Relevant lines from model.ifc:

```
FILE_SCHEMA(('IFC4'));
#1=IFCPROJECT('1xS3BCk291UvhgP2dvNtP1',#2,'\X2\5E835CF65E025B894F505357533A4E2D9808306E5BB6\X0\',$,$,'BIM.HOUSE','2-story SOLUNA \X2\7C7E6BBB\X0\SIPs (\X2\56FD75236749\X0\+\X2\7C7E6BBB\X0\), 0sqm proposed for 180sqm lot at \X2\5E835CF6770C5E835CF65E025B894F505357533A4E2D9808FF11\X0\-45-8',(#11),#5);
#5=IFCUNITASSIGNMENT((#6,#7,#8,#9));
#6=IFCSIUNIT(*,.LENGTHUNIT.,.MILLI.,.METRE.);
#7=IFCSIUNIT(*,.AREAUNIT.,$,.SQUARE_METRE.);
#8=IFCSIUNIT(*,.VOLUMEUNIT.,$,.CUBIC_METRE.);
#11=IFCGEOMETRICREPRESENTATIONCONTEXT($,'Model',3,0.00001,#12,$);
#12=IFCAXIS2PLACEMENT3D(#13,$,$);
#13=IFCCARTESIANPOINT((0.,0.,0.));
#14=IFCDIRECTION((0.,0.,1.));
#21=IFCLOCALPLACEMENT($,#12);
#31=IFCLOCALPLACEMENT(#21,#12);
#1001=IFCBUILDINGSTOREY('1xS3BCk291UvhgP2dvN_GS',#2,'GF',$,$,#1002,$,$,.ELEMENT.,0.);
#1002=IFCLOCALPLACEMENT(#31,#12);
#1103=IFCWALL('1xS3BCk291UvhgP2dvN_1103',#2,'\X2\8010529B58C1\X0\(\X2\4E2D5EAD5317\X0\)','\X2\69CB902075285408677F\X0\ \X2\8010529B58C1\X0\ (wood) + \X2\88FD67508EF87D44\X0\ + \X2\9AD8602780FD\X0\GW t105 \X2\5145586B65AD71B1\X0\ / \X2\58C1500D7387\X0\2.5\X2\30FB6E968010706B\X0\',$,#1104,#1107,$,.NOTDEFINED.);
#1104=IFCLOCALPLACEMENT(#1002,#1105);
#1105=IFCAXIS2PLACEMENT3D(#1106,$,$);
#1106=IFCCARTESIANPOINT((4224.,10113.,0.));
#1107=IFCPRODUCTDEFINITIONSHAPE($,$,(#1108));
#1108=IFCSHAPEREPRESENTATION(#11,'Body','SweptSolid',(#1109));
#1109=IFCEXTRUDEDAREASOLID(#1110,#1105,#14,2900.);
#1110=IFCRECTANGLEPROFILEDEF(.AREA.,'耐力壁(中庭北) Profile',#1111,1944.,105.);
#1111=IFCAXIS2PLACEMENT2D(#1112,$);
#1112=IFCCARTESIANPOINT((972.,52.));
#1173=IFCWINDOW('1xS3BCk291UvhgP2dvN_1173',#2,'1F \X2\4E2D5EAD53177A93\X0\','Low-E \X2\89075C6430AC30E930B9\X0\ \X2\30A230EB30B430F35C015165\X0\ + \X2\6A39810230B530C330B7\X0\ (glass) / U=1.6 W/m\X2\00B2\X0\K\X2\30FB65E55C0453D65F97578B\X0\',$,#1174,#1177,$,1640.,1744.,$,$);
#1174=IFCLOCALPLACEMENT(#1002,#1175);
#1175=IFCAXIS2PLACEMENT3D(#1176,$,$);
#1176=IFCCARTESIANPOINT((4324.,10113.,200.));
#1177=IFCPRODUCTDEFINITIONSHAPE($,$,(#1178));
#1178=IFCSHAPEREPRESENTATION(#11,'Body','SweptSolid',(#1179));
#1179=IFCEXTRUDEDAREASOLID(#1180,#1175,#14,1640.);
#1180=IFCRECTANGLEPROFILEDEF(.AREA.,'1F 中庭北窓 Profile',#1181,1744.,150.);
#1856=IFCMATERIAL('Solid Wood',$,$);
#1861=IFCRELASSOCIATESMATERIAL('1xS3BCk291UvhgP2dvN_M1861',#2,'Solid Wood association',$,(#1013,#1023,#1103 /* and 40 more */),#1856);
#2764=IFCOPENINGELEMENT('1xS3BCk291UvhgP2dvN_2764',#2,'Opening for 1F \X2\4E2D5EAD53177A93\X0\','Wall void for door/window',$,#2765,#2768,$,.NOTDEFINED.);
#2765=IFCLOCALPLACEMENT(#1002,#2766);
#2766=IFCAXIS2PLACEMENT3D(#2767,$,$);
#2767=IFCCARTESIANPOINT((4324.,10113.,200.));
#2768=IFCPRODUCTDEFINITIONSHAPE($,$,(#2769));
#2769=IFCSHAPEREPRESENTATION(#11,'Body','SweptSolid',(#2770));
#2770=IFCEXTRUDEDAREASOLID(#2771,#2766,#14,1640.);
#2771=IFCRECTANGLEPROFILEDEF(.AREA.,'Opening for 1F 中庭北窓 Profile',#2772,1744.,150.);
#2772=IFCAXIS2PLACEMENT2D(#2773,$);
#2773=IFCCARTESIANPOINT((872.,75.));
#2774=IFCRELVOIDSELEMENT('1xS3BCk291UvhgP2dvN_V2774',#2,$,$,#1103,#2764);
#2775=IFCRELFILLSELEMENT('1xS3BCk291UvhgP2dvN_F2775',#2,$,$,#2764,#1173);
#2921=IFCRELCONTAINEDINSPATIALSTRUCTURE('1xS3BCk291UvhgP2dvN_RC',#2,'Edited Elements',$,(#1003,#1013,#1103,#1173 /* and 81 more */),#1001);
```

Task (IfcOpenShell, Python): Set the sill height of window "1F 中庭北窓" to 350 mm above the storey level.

```python
import numpy as np
import ifcopenshell
import ifcopenshell.api.geometry
import ifcopenshell.geom
import ifcopenshell.util.element
import ifcopenshell.util.placement
import ifcopenshell.util.shape
import ifcopenshell.util.unit

model = ifcopenshell.open("model.ifc")
unit_scale = ifcopenshell.util.unit.calculate_unit_scale(model)

window = model.by_id(1173)
opening = window.FillsVoids[0].RelatingOpeningElement
storey = ifcopenshell.util.element.get_container(window, ifc_class="IfcBuildingStorey")
level = ifcopenshell.util.placement.get_local_placement(storey.ObjectPlacement)[2, 3]

# The opening's origin need not be at the sill, so measure its lowest point.
shape = ifcopenshell.geom.create_shape(ifcopenshell.geom.settings(), opening)
bottom = ifcopenshell.util.shape.get_shape_bottom_elevation(shape, shape.geometry) / unit_scale
dz = level + 0.35 / unit_scale - bottom

shift = np.array([0.0, 0.0, dz])
# The window is not placed relative to its opening, so move both.
for product in (opening, window):
    matrix = ifcopenshell.util.placement.get_local_placement(product.ObjectPlacement)
    matrix[:3, 3] += shift
    ifcopenshell.api.geometry.edit_object_placement(model, product=product, matrix=matrix, is_si=False)

print(f"moved by {dz * unit_scale:+.3f} m")

model.write("model-out.ifc")
```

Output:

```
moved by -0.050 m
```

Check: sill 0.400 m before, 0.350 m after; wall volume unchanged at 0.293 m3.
